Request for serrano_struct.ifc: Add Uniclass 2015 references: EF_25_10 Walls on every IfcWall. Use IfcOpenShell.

First a look at what the model holds.

```python
import ifcopenshell

model = ifcopenshell.open("serrano_struct.ifc")
print(model.schema)
print("classifications:", [c.Name for c in model.by_type("IfcClassification")])
for ifc_class in ("IfcDoor", "IfcRoof", "IfcStair", "IfcWall", "IfcWindow"):
    print(ifc_class, len(model.by_type(ifc_class)))
```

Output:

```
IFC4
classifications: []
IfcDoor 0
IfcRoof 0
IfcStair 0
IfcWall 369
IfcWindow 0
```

```python
import ifcopenshell
import ifcopenshell.api.classification

model = ifcopenshell.open("serrano_struct.ifc")

system = ifcopenshell.api.classification.add_classification(model, classification="Uniclass 2015")

codes = {
    "IfcWall": ("EF_25_10", "Walls"),
}
for ifc_class, (code, name) in codes.items():
    products = model.by_type(ifc_class)
    ifcopenshell.api.classification.add_reference(
        model, products=products, classification=system, identification=code, name=name
    )
    print(code, len(products))

model.write("serrano_struct_updated.ifc")
```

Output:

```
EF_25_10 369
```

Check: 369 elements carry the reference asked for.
